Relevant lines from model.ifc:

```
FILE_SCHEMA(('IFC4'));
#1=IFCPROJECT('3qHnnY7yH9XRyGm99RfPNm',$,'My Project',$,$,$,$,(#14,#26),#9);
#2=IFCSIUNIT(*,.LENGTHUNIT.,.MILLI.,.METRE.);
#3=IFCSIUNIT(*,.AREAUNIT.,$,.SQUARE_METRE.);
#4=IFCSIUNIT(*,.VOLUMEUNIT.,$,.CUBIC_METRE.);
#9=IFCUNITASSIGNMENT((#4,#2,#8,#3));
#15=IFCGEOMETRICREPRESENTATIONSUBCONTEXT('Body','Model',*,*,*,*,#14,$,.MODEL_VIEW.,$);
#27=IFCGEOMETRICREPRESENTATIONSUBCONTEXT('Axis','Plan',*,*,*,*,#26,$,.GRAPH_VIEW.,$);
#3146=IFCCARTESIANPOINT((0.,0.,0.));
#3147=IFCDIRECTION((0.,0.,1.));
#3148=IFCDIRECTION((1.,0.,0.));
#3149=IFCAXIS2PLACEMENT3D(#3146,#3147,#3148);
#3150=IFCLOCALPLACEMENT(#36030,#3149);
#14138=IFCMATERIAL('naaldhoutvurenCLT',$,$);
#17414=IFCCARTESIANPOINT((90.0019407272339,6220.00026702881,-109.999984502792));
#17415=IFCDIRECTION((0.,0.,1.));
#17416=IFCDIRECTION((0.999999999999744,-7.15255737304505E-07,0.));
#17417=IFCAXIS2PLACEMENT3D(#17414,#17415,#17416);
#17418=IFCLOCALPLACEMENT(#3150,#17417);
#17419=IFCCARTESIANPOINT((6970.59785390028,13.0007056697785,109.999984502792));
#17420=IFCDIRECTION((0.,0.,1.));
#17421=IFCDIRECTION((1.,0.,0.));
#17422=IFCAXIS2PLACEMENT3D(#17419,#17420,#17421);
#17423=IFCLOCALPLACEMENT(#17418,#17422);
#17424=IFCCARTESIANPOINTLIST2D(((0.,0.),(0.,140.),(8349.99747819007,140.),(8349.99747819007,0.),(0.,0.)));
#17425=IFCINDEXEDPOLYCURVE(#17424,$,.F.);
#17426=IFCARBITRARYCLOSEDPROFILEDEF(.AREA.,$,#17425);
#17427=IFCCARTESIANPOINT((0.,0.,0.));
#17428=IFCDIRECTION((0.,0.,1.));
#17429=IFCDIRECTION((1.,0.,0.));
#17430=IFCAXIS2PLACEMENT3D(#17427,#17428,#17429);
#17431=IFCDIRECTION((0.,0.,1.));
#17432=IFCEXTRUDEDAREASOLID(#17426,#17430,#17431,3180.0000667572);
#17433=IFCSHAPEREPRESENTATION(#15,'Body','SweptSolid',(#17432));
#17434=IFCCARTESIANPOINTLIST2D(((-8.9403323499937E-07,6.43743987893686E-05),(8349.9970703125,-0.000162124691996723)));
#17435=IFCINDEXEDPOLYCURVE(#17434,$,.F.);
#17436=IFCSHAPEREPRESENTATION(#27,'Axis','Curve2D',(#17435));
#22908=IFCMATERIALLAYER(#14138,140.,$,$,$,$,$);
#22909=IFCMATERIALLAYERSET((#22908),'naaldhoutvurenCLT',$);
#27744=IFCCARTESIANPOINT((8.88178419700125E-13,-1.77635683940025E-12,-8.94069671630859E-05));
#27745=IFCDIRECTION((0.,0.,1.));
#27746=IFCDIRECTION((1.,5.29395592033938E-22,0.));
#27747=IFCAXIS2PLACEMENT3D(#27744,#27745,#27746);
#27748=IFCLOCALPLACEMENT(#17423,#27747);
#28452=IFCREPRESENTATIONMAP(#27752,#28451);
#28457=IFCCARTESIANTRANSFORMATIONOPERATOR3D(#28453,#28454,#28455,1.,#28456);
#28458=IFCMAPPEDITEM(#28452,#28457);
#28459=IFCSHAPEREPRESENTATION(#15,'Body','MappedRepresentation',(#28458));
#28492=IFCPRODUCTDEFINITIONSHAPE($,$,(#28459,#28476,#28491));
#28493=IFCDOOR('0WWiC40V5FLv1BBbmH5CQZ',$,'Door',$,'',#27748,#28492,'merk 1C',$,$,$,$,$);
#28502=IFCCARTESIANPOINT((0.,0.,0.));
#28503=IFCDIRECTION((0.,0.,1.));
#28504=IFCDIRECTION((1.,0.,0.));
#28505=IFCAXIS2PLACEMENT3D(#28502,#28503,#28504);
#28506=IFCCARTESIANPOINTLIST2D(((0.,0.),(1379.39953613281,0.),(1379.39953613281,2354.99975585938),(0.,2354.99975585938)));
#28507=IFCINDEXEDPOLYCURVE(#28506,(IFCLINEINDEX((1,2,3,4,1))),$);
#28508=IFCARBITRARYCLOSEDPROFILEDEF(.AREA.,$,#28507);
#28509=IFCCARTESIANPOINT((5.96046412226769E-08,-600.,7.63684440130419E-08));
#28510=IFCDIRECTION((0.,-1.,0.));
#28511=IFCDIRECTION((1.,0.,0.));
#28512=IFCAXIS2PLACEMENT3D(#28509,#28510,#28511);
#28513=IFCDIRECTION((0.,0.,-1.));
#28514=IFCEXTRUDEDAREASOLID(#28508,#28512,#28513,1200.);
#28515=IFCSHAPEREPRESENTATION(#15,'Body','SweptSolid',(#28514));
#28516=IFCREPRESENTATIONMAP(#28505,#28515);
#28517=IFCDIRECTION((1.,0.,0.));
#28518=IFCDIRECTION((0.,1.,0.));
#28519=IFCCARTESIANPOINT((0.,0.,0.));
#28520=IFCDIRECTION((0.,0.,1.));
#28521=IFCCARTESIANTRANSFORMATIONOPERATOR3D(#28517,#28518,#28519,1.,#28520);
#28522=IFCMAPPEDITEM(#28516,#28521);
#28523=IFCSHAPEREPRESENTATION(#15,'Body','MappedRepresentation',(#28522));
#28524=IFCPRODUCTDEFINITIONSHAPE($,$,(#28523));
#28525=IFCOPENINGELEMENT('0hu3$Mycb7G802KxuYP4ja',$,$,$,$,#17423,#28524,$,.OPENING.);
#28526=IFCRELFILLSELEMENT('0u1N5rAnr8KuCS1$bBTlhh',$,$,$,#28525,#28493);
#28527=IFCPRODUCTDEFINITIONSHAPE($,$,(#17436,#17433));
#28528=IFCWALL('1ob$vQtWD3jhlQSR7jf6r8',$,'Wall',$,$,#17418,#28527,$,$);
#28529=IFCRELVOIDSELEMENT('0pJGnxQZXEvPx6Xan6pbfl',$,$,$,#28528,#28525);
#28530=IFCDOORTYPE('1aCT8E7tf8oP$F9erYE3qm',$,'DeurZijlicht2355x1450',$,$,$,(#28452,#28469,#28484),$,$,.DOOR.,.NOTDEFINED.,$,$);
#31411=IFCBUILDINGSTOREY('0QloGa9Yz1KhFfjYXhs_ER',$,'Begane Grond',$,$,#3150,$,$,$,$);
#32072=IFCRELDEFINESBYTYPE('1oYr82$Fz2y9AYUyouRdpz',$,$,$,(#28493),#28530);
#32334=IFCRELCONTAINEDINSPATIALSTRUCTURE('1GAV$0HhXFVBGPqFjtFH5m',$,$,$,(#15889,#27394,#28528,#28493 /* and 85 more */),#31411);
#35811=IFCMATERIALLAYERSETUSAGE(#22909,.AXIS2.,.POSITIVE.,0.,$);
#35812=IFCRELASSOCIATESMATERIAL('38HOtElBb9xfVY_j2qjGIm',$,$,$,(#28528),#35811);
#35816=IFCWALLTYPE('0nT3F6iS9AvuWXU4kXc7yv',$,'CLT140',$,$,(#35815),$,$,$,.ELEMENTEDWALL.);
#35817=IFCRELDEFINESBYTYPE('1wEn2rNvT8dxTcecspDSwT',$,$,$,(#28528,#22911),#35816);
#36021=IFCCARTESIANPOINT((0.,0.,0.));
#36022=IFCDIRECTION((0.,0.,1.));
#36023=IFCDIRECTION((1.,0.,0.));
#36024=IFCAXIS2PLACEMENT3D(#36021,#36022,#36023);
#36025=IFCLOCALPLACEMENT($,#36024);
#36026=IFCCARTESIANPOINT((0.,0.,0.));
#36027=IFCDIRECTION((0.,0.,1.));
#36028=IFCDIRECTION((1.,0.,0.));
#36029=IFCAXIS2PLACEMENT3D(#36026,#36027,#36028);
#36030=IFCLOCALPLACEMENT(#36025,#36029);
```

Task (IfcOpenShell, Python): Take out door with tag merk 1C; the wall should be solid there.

```python
import ifcopenshell
import ifcopenshell.api.feature
import ifcopenshell.api.root
import ifcopenshell.geom
import ifcopenshell.util.shape

model = ifcopenshell.open("model.ifc")
settings = ifcopenshell.geom.settings()


def volume(element):
    """Net volume in cubic metres, openings subtracted."""
    shape = ifcopenshell.geom.create_shape(settings, element)
    return ifcopenshell.util.shape.get_volume(shape.geometry)


door = model.by_id(28493)
opening = door.FillsVoids[0].RelatingOpeningElement
wall = opening.VoidsElements[0].RelatingBuildingElement
before = volume(wall)

ifcopenshell.api.root.remove_product(model, product=door)
ifcopenshell.api.feature.remove_feature(model, feature=opening)

after = volume(wall)

print(f"wall volume {before:.3f} -> {after:.3f} m3")

model.write("model_rev.ifc")
```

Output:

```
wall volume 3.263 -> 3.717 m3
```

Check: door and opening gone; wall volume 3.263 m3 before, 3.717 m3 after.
